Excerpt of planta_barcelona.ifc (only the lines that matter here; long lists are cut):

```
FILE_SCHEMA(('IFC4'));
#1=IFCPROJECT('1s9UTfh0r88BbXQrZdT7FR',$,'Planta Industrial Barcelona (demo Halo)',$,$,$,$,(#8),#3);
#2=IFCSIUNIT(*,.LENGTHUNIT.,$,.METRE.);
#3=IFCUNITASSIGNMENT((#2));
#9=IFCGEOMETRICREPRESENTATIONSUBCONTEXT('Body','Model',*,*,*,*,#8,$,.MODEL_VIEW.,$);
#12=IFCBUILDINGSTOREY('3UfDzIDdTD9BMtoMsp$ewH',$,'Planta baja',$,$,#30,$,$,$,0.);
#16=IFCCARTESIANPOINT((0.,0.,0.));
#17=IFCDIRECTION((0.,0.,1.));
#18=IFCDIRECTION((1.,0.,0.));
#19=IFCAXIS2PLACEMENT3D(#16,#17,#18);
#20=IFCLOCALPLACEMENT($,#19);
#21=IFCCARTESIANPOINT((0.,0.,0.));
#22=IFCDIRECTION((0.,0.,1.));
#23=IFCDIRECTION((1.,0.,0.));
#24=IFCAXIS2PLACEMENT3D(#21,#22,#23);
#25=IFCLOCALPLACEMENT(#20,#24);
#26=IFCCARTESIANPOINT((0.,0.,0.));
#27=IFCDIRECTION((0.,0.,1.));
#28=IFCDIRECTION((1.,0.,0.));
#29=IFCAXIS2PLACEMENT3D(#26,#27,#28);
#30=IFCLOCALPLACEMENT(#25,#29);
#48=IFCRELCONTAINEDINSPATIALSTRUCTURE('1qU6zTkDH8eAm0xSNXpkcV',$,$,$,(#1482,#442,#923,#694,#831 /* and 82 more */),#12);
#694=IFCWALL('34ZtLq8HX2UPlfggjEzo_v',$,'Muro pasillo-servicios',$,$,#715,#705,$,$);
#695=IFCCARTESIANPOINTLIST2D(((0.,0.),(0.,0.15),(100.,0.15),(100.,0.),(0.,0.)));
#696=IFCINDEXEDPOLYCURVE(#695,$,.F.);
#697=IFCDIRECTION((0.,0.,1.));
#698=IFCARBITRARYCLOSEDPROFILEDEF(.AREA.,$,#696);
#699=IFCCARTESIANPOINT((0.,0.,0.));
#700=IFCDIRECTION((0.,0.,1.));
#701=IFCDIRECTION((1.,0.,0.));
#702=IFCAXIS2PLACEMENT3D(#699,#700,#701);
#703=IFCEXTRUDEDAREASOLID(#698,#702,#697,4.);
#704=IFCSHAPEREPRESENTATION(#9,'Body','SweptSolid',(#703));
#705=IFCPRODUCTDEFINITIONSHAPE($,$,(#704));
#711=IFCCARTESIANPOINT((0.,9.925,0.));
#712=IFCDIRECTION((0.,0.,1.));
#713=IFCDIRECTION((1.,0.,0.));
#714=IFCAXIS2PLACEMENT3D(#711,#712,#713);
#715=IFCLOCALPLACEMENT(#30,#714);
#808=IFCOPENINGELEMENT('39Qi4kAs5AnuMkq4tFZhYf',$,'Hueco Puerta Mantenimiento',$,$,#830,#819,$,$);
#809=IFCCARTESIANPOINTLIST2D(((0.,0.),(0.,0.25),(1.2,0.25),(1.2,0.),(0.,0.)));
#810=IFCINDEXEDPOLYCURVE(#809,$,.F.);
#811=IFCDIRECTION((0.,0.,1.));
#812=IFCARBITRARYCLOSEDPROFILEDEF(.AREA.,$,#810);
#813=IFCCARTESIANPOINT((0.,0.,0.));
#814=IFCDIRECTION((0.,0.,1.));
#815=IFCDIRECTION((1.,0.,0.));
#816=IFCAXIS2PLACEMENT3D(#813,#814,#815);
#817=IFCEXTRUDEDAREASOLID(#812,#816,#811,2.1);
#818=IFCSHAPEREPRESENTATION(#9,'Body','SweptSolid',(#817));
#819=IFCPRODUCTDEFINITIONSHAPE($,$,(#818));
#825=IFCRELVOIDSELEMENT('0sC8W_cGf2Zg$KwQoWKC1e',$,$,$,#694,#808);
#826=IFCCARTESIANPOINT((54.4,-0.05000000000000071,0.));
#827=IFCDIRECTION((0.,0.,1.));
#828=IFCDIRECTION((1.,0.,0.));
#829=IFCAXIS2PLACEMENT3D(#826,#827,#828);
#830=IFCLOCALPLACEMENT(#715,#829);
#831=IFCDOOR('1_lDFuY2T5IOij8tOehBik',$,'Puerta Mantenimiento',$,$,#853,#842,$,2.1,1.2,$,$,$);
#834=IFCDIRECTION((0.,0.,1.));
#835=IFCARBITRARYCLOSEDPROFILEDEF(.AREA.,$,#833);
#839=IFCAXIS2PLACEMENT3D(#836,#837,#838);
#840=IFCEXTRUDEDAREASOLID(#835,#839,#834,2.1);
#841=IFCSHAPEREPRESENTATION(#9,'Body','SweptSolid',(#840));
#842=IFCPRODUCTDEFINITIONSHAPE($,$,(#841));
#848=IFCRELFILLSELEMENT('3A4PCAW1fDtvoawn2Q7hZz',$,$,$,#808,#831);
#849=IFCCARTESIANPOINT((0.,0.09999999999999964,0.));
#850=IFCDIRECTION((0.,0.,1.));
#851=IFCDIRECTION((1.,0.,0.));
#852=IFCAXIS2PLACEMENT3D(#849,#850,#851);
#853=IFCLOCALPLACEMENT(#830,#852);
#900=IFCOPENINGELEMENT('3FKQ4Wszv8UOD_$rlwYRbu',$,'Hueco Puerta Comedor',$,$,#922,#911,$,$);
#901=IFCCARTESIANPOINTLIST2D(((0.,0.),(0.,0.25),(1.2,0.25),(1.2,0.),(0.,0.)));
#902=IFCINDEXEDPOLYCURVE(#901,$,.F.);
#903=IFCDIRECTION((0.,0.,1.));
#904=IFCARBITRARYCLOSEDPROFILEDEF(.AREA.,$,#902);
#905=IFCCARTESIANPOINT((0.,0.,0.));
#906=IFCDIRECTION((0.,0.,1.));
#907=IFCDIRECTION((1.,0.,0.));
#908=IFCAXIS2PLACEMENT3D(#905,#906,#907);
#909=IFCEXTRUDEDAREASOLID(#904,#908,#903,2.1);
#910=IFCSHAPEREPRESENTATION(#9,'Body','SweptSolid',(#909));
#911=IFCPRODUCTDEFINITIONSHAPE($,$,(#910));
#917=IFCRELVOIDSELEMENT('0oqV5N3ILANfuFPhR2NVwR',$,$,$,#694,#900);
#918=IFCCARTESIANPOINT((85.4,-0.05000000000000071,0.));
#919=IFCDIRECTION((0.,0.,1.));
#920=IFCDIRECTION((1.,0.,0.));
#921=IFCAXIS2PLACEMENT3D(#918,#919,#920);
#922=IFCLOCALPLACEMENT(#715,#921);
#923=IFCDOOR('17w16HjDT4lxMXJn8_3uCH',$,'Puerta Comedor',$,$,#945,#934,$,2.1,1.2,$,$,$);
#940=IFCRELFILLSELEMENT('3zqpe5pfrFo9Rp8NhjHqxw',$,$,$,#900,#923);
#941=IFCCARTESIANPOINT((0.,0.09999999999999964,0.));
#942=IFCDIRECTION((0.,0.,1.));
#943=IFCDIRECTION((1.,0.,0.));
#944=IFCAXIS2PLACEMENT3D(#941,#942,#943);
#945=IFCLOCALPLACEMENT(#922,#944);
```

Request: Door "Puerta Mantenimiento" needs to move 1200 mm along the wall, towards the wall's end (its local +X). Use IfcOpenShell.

```python
import ifcopenshell
import ifcopenshell.api.geometry
import ifcopenshell.util.placement

model = ifcopenshell.open("planta_barcelona.ifc")

door = model.by_guid("1_lDFuY2T5IOij8tOehBik")
opening = door.FillsVoids[0].RelatingOpeningElement
wall = opening.VoidsElements[0].RelatingBuildingElement

wall_matrix = ifcopenshell.util.placement.get_local_placement(wall.ObjectPlacement)
shift = wall_matrix[:3, 0] * 1.2
before = ifcopenshell.util.placement.get_local_placement(door.ObjectPlacement)[:3, 3].copy()

# The door is placed relative to its opening, so it follows when the opening moves.
matrix = ifcopenshell.util.placement.get_local_placement(opening.ObjectPlacement)
matrix[:3, 3] += shift
ifcopenshell.api.geometry.edit_object_placement(
    model, product=opening, matrix=matrix, is_si=False, should_transform_children=True
)

after = ifcopenshell.util.placement.get_local_placement(door.ObjectPlacement)[:3, 3]
print("door moved by", (after - before).round(3) + 0.0)

model.write("planta_barcelona_edited.ifc")
```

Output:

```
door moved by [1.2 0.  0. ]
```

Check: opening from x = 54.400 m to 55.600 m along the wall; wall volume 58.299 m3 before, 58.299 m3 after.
